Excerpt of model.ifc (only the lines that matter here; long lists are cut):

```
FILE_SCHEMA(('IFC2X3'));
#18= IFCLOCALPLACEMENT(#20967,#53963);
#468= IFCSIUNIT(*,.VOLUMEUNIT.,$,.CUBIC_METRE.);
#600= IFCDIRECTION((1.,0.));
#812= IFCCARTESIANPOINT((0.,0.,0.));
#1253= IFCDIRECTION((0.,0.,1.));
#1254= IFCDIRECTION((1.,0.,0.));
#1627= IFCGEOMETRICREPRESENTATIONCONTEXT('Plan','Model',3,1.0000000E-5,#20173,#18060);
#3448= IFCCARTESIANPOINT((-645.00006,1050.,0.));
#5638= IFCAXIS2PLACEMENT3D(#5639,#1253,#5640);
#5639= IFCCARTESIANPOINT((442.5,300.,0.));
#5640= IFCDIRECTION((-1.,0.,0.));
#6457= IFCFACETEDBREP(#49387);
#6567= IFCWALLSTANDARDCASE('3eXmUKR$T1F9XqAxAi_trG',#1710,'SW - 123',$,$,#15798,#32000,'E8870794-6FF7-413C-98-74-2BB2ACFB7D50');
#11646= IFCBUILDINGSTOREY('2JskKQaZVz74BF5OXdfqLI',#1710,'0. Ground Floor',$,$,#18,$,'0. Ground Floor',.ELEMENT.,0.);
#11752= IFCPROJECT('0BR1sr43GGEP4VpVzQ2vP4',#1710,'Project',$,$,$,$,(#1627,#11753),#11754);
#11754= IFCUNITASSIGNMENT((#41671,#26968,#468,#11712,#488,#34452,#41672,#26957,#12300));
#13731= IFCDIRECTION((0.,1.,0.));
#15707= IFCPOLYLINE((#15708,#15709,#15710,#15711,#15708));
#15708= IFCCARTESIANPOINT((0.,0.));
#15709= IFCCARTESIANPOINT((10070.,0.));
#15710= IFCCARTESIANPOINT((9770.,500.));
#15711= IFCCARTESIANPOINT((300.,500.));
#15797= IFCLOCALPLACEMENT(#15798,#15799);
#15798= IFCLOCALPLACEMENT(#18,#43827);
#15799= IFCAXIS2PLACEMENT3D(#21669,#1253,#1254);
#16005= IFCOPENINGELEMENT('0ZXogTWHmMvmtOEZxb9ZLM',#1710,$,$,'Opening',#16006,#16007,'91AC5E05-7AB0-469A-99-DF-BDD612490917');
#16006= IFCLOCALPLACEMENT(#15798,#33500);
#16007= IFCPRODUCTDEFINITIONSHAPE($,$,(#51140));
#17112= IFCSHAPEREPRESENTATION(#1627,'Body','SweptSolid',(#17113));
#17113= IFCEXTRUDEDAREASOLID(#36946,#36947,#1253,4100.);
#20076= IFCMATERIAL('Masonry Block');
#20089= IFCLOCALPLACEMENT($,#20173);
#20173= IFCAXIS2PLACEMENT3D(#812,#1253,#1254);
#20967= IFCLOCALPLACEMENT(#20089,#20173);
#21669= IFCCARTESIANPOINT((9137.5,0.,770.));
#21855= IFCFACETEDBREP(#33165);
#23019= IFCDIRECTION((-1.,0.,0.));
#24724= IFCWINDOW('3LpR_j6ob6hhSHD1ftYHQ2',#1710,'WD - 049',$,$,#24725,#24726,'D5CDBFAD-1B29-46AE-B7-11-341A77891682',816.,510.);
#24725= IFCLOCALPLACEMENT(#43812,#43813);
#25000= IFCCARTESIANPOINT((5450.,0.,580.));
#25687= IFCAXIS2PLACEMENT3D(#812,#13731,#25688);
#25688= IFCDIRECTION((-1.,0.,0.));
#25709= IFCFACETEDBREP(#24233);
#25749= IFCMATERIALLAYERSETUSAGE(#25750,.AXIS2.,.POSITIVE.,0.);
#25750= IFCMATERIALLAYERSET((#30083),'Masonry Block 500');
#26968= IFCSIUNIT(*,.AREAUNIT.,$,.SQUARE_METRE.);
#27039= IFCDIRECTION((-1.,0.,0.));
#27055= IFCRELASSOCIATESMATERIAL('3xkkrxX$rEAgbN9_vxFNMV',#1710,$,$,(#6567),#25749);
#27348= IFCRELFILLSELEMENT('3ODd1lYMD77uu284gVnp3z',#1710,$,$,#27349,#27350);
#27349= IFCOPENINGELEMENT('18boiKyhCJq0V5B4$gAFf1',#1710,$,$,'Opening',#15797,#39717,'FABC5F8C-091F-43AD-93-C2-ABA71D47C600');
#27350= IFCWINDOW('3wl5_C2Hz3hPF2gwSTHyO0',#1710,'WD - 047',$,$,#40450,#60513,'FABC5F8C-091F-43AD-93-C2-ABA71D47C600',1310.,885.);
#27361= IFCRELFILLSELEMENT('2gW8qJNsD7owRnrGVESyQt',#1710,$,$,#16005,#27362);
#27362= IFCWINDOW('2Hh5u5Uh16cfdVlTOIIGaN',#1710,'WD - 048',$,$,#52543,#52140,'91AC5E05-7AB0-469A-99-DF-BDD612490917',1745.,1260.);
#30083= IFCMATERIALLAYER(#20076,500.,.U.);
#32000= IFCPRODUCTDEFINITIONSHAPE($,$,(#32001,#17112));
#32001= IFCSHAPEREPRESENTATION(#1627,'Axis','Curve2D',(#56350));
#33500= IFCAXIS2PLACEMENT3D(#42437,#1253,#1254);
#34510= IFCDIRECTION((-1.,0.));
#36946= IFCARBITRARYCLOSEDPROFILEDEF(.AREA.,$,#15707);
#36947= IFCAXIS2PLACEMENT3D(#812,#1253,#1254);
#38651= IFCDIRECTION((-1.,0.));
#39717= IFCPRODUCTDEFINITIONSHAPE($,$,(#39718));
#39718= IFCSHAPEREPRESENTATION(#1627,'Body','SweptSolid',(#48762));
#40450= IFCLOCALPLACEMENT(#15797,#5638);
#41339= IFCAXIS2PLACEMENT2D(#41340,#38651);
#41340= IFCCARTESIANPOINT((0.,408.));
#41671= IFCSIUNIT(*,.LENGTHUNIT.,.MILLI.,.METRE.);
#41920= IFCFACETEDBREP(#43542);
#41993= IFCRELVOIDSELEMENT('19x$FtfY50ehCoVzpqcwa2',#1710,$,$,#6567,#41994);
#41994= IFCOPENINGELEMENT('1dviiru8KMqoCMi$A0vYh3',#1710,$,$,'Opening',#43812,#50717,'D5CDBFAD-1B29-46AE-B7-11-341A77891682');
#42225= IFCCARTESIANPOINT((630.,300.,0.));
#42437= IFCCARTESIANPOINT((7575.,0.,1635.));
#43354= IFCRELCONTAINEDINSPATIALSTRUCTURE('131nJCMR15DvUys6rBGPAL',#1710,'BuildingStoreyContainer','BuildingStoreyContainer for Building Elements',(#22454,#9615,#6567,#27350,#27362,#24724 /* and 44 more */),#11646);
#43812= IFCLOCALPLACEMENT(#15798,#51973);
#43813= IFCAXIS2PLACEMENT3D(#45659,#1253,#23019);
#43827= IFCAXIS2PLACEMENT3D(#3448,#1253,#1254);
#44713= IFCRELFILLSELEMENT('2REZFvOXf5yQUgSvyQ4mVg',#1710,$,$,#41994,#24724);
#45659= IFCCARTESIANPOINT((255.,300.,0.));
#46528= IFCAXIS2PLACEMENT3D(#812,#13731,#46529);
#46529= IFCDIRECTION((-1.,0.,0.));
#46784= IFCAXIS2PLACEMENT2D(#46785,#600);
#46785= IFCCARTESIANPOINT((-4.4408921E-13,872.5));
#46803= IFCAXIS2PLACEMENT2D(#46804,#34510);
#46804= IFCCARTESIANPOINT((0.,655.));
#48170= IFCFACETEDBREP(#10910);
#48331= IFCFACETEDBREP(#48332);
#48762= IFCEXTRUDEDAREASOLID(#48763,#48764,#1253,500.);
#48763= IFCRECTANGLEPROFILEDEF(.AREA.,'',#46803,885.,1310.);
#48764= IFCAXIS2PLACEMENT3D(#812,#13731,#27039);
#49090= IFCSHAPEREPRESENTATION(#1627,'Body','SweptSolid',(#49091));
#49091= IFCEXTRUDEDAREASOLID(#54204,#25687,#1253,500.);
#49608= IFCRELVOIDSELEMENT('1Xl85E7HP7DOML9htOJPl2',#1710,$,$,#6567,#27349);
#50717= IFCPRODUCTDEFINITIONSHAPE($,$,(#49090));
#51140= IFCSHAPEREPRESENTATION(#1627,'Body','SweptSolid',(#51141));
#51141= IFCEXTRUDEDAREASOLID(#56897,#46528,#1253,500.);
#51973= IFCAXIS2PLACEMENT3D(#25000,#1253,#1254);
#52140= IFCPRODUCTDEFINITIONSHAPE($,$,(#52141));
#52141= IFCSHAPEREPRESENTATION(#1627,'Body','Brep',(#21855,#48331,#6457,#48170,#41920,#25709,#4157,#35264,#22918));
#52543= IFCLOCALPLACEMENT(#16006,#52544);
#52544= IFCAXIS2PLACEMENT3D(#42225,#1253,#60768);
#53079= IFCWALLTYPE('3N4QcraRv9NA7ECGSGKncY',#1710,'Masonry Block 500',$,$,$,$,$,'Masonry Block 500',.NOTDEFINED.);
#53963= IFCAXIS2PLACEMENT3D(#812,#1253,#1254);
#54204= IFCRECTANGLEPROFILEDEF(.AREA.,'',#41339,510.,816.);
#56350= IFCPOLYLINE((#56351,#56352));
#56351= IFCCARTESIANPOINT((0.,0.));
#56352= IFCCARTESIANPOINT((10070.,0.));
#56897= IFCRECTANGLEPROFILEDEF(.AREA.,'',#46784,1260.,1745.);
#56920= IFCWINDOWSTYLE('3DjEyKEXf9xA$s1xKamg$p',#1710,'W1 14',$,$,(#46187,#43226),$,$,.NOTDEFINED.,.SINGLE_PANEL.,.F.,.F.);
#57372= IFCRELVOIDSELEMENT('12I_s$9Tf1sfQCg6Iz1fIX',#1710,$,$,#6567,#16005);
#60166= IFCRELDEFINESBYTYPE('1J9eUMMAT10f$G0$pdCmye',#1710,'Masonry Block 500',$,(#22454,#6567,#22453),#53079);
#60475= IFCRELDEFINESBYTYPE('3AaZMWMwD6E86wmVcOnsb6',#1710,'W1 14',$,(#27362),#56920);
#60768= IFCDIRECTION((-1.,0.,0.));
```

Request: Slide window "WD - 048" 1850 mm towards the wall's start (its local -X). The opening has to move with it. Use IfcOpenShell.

```python
import ifcopenshell
import ifcopenshell.api.geometry
import ifcopenshell.util.placement

model = ifcopenshell.open("model.ifc")

window = model.by_guid("2Hh5u5Uh16cfdVlTOIIGaN")
opening = window.FillsVoids[0].RelatingOpeningElement
wall = opening.VoidsElements[0].RelatingBuildingElement

wall_matrix = ifcopenshell.util.placement.get_local_placement(wall.ObjectPlacement)
shift = wall_matrix[:3, 0] * -1850.0
before = ifcopenshell.util.placement.get_local_placement(window.ObjectPlacement)[:3, 3].copy()

# The window is placed relative to its opening, so it follows when the opening moves.
matrix = ifcopenshell.util.placement.get_local_placement(opening.ObjectPlacement)
matrix[:3, 3] += shift
ifcopenshell.api.geometry.edit_object_placement(
    model, product=opening, matrix=matrix, is_si=False, should_transform_children=True
)

after = ifcopenshell.util.placement.get_local_placement(window.ObjectPlacement)[:3, 3]
print("window moved by", (after - before).round(3) + 0.0)

model.write("model_v2.ifc")
```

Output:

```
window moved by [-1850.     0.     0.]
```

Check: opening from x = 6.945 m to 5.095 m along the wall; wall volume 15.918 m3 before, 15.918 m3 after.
